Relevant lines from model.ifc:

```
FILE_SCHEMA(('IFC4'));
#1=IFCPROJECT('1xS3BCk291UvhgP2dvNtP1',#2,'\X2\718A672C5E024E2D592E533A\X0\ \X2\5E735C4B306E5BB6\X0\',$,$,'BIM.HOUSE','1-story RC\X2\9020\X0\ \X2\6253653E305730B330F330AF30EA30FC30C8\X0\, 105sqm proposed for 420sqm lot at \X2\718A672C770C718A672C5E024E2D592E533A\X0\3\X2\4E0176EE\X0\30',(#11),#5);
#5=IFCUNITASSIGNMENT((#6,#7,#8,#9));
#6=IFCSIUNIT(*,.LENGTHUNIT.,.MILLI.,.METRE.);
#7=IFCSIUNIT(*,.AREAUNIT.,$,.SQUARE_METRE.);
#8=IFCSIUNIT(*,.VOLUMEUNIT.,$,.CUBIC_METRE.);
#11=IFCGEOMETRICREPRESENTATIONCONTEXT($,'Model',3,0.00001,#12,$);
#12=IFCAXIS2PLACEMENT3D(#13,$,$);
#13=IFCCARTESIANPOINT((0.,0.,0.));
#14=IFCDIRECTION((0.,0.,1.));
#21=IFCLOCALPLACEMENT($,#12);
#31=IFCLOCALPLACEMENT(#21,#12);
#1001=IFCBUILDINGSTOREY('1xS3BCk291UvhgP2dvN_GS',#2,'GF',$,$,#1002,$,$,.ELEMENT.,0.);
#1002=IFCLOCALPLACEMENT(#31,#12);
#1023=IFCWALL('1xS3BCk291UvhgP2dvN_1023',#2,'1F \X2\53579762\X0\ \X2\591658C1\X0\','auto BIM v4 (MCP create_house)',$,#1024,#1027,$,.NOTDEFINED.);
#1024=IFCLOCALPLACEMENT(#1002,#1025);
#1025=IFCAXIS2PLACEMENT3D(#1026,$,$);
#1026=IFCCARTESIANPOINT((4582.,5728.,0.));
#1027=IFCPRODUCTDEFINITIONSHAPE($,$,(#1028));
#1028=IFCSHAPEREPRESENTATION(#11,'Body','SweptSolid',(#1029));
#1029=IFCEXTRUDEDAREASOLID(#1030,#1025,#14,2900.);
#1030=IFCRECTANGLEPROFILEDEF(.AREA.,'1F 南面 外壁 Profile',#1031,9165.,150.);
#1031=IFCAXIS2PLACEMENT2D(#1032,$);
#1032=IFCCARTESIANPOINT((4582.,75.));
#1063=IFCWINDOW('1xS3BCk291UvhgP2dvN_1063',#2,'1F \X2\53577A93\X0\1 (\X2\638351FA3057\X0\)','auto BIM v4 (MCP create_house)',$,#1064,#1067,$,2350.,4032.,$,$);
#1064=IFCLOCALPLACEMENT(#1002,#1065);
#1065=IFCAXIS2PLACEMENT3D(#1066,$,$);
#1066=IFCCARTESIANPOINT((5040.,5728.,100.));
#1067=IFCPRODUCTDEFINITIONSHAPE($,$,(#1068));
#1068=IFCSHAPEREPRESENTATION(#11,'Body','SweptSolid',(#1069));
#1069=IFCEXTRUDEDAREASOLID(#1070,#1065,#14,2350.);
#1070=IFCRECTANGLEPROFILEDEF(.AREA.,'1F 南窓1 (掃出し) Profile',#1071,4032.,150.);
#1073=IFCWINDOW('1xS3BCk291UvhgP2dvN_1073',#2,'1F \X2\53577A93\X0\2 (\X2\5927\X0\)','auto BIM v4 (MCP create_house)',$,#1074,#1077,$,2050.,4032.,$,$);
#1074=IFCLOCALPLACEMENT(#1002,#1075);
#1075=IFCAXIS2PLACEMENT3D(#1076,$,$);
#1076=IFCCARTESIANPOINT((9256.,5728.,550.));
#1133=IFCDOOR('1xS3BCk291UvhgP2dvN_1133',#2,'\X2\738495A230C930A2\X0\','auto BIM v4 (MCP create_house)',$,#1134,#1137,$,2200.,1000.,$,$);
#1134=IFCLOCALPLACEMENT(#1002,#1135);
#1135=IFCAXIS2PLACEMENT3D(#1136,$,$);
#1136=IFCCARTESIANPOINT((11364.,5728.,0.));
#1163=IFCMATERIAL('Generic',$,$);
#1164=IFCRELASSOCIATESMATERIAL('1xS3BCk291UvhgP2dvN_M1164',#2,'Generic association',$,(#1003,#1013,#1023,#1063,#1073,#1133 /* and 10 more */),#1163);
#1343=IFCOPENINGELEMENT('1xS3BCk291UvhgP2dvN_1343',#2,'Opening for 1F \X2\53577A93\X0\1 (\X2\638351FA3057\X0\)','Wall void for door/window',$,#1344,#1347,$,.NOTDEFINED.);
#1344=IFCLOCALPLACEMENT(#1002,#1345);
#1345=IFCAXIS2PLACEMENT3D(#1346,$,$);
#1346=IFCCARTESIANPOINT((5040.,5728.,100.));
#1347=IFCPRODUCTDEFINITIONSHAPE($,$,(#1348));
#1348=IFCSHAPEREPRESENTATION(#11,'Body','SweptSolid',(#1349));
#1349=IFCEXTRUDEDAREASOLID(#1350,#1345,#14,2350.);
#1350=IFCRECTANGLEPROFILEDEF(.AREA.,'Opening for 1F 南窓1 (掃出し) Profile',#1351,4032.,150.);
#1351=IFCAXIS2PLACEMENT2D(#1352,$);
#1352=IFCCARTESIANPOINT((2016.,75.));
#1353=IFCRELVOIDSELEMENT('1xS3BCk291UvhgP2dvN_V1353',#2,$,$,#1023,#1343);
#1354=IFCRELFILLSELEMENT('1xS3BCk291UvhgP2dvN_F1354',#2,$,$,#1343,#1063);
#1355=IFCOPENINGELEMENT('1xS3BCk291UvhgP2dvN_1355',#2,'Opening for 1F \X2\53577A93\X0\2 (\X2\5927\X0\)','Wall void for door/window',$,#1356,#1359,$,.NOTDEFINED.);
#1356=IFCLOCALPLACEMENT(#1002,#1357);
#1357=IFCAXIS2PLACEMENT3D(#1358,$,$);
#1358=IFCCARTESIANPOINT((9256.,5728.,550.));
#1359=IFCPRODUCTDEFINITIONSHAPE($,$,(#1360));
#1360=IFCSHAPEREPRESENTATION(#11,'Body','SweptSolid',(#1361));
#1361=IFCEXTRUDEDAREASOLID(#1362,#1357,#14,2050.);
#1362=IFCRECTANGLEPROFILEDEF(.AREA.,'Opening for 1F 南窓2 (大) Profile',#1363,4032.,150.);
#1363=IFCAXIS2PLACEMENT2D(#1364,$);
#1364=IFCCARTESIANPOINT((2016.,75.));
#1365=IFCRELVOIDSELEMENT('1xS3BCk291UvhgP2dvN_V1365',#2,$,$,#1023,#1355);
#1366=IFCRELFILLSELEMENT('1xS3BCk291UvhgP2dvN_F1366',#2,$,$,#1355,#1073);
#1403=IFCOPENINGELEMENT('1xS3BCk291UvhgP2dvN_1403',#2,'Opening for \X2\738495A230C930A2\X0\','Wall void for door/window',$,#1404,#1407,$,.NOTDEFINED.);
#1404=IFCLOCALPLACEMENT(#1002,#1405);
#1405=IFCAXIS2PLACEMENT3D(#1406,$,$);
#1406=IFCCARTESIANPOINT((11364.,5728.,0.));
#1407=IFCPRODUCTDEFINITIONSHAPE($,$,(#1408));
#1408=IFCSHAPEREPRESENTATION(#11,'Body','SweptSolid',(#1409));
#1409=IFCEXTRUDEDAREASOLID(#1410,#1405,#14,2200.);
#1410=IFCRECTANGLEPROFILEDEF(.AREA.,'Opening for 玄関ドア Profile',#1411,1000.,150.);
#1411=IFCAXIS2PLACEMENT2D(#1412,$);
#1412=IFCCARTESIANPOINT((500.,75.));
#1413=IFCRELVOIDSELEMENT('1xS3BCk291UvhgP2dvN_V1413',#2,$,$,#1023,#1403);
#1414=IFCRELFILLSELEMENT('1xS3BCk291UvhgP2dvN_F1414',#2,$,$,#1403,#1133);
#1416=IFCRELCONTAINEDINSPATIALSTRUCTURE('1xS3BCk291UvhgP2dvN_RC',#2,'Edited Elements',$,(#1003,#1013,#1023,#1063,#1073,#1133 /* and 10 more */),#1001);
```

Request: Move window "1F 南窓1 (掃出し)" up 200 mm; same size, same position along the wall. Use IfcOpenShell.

```python
import numpy as np
import ifcopenshell
import ifcopenshell.api.geometry
import ifcopenshell.util.placement
import ifcopenshell.util.unit

model = ifcopenshell.open("model.ifc")
unit_scale = ifcopenshell.util.unit.calculate_unit_scale(model)

window = model.by_guid("1xS3BCk291UvhgP2dvN_1063")
opening = window.FillsVoids[0].RelatingOpeningElement
dz = 200.0

shift = np.array([0.0, 0.0, dz])
# The window is not placed relative to its opening, so move both.
for product in (opening, window):
    matrix = ifcopenshell.util.placement.get_local_placement(product.ObjectPlacement)
    matrix[:3, 3] += shift
    ifcopenshell.api.geometry.edit_object_placement(model, product=product, matrix=matrix, is_si=False)

print(f"moved by {dz * unit_scale:+.3f} m")

model.write("model-out.ifc")
```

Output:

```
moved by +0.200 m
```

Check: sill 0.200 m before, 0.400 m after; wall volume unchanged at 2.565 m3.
